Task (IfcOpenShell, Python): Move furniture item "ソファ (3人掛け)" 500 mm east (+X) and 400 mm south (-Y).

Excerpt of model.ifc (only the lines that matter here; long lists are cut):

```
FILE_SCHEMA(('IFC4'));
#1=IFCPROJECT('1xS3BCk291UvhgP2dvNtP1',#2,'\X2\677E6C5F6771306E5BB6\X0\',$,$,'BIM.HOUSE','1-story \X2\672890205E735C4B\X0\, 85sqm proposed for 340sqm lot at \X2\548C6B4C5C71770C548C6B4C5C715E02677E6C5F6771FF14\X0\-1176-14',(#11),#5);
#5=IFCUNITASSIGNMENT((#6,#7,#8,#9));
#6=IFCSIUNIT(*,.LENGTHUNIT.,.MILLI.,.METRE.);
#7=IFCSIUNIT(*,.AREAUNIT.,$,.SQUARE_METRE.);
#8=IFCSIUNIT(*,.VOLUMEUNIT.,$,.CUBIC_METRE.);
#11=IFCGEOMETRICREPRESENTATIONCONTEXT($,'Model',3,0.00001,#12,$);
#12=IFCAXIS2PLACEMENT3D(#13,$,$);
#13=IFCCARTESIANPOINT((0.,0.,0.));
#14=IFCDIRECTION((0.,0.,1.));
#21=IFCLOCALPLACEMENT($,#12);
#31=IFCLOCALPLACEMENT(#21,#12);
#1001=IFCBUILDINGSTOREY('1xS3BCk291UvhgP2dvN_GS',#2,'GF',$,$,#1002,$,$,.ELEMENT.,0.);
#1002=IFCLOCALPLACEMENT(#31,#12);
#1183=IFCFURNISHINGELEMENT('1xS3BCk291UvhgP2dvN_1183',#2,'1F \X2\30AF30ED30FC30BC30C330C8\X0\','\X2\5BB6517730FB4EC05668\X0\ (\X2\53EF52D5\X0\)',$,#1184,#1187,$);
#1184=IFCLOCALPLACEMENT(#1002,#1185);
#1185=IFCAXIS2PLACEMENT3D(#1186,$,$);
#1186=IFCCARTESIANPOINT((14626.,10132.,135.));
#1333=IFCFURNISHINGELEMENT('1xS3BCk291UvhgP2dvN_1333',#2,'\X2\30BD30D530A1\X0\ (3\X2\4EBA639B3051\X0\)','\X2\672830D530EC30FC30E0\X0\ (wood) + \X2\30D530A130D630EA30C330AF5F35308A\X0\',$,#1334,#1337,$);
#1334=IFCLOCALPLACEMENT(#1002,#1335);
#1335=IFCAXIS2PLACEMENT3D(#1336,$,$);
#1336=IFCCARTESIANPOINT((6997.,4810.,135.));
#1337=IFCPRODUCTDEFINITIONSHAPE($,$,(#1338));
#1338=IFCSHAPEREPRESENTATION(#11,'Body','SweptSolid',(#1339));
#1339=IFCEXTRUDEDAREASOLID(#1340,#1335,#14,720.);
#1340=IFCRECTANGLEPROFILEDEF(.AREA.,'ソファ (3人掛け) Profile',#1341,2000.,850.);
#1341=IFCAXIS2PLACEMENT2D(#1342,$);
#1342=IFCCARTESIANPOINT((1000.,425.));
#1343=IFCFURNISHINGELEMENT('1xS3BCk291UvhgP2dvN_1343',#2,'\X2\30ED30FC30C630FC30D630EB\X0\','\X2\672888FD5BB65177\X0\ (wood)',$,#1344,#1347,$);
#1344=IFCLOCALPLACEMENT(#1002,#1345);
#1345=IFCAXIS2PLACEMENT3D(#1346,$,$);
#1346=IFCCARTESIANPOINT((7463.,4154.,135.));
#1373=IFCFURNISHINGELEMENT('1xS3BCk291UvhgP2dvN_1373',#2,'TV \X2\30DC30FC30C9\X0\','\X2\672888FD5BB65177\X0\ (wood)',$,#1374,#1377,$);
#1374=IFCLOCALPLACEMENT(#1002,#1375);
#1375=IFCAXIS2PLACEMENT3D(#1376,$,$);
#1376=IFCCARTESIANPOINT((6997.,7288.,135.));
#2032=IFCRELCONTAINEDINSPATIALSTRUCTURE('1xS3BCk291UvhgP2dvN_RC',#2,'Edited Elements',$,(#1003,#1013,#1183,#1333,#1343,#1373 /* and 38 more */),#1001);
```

```python
import ifcopenshell
import ifcopenshell.api.geometry
import ifcopenshell.util.placement
import ifcopenshell.util.unit

model = ifcopenshell.open("model.ifc")
unit_scale = ifcopenshell.util.unit.calculate_unit_scale(model)

item = model.by_guid("1xS3BCk291UvhgP2dvN_1333")
matrix = ifcopenshell.util.placement.get_local_placement(item.ObjectPlacement)
matrix[0, 3] += 0.5 / unit_scale
matrix[1, 3] -= 0.4 / unit_scale
ifcopenshell.api.geometry.edit_object_placement(model, product=item, matrix=matrix, is_si=False)

print(ifcopenshell.util.placement.get_local_placement(item.ObjectPlacement).round(3) + 0.0)

model.write("model_edited.ifc")
```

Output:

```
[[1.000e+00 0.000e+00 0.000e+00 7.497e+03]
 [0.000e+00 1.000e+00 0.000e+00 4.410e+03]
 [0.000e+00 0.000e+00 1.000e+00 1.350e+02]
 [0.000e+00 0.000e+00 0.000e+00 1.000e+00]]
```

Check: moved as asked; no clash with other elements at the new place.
